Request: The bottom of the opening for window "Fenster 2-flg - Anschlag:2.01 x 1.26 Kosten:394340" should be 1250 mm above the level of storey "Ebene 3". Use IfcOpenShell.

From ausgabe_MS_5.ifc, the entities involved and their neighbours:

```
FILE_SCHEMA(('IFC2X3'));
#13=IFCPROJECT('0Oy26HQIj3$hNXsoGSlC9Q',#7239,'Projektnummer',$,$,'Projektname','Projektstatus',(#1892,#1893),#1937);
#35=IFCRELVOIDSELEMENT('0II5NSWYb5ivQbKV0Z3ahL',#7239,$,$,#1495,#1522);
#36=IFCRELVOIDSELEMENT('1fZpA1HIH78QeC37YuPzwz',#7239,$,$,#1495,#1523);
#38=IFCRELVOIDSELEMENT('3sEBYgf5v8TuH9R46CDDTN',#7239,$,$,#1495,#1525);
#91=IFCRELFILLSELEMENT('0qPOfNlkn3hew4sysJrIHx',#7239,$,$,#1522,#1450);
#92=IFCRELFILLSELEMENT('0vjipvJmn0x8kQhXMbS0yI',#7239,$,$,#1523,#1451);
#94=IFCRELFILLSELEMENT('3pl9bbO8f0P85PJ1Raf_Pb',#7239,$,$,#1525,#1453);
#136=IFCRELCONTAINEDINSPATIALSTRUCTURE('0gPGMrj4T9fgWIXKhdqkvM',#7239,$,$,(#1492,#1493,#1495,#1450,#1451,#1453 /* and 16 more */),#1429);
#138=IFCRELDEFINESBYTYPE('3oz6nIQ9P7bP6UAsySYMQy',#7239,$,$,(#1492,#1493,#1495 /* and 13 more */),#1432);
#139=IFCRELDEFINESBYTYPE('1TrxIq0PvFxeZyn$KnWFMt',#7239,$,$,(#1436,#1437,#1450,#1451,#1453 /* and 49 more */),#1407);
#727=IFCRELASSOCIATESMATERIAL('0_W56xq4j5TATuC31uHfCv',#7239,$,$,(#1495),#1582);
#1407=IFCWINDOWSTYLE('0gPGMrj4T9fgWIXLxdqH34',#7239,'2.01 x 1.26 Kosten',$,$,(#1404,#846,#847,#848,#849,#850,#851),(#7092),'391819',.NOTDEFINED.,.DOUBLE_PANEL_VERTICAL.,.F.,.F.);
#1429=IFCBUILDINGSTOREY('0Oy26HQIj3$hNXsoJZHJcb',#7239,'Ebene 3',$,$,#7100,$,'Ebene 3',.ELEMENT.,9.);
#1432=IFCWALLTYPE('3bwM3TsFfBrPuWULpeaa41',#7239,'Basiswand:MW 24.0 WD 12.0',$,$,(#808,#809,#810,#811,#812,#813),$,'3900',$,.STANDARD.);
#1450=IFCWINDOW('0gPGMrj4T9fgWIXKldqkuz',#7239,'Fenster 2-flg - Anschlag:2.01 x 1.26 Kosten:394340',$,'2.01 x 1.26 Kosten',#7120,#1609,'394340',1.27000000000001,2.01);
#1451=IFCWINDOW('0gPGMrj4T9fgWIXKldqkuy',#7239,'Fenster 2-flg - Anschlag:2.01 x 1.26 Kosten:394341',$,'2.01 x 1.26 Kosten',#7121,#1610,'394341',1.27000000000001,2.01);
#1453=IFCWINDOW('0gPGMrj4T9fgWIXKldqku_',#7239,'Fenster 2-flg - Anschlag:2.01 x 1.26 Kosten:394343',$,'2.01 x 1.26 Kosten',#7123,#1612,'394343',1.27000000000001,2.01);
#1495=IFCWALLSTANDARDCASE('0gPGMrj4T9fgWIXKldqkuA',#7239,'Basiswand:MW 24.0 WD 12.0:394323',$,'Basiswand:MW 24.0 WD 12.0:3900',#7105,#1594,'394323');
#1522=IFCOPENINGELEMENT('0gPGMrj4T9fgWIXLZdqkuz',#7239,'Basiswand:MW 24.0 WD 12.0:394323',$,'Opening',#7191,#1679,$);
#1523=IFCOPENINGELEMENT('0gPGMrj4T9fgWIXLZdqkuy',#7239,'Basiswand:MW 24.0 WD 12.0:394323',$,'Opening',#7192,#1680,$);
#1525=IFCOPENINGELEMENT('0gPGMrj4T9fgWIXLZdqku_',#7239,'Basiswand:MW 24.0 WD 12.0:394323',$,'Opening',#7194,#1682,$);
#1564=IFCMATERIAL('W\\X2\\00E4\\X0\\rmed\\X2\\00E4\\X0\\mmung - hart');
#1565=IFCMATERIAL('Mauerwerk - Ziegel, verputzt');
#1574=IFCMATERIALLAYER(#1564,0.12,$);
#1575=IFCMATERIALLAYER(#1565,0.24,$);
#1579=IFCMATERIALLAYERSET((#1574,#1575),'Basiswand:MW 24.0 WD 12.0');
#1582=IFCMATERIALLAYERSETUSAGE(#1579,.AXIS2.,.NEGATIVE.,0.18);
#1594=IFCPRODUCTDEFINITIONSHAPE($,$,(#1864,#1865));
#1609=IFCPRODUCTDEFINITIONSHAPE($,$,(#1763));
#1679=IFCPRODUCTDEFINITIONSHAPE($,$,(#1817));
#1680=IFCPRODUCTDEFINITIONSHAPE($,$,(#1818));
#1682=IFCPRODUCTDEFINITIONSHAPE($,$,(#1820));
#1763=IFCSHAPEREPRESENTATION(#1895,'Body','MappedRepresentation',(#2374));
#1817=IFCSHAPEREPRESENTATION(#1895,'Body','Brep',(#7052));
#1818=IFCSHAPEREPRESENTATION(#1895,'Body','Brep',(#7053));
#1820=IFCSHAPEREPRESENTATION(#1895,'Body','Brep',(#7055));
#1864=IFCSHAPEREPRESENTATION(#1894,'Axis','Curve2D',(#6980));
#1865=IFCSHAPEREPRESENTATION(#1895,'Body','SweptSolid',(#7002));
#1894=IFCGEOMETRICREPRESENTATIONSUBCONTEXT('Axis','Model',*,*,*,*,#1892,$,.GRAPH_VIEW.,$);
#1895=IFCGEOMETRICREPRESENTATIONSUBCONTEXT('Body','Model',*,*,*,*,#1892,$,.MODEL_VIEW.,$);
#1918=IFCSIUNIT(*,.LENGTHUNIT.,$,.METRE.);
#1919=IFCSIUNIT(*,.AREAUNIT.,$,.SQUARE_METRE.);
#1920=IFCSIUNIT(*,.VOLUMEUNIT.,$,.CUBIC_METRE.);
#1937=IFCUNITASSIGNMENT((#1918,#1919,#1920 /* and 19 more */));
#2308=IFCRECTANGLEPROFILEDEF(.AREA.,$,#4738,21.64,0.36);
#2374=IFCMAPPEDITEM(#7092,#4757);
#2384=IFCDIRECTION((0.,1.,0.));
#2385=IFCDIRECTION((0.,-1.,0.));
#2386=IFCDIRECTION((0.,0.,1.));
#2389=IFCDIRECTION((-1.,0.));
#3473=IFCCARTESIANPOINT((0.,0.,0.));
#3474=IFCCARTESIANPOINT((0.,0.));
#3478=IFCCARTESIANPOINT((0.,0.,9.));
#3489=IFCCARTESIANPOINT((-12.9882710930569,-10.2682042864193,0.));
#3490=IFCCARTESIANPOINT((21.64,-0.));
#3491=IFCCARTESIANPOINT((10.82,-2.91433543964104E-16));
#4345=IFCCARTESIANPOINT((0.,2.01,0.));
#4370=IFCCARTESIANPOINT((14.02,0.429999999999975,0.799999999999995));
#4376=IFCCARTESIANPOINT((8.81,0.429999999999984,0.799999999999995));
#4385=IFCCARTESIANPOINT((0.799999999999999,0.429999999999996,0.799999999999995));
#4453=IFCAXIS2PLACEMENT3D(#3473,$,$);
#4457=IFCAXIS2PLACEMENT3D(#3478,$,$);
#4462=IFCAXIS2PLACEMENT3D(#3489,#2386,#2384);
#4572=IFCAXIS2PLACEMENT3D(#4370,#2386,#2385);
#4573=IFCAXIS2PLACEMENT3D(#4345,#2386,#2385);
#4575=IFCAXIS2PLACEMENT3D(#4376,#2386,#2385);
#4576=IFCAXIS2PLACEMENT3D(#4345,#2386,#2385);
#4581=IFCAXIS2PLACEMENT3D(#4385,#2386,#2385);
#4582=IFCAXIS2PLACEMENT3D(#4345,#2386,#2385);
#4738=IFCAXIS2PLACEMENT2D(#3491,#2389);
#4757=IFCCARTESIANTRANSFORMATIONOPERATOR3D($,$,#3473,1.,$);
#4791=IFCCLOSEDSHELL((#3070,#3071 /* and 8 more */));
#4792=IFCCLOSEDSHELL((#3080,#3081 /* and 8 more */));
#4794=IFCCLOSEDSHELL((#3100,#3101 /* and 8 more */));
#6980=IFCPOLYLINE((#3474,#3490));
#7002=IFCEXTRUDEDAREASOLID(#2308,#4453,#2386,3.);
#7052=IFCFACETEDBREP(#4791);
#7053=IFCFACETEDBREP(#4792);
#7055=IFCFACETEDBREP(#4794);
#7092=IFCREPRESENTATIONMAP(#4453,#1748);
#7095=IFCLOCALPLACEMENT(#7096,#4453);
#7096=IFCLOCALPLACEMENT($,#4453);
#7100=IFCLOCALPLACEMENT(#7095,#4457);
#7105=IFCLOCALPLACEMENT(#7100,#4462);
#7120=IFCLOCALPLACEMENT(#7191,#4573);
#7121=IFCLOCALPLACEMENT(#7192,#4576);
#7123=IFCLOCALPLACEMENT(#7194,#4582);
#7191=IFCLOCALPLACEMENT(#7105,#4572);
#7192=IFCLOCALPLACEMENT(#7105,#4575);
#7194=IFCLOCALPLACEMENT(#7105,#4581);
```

```python
import numpy as np
import ifcopenshell
import ifcopenshell.api.geometry
import ifcopenshell.geom
import ifcopenshell.util.element
import ifcopenshell.util.placement
import ifcopenshell.util.shape
import ifcopenshell.util.unit

model = ifcopenshell.open("ausgabe_MS_5.ifc")
unit_scale = ifcopenshell.util.unit.calculate_unit_scale(model)

window = model.by_guid("0gPGMrj4T9fgWIXKldqkuz")
opening = window.FillsVoids[0].RelatingOpeningElement
storey = ifcopenshell.util.element.get_container(window, ifc_class="IfcBuildingStorey")
level = ifcopenshell.util.placement.get_local_placement(storey.ObjectPlacement)[2, 3]

# The opening's origin need not be at the sill, so measure its lowest point.
shape = ifcopenshell.geom.create_shape(ifcopenshell.geom.settings(), opening)
bottom = ifcopenshell.util.shape.get_shape_bottom_elevation(shape, shape.geometry) / unit_scale
dz = level + 1.25 / unit_scale - bottom

shift = np.array([0.0, 0.0, dz])
# The window is placed relative to its opening, so it follows when the opening moves.
matrix = ifcopenshell.util.placement.get_local_placement(opening.ObjectPlacement)
matrix[:3, 3] += shift
ifcopenshell.api.geometry.edit_object_placement(
    model, product=opening, matrix=matrix, is_si=False, should_transform_children=True
)

print(f"moved by {dz * unit_scale:+.3f} m")

model.write("ausgabe_MS_5_v2.ifc")
```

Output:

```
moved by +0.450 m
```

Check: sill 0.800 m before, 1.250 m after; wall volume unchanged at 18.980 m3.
